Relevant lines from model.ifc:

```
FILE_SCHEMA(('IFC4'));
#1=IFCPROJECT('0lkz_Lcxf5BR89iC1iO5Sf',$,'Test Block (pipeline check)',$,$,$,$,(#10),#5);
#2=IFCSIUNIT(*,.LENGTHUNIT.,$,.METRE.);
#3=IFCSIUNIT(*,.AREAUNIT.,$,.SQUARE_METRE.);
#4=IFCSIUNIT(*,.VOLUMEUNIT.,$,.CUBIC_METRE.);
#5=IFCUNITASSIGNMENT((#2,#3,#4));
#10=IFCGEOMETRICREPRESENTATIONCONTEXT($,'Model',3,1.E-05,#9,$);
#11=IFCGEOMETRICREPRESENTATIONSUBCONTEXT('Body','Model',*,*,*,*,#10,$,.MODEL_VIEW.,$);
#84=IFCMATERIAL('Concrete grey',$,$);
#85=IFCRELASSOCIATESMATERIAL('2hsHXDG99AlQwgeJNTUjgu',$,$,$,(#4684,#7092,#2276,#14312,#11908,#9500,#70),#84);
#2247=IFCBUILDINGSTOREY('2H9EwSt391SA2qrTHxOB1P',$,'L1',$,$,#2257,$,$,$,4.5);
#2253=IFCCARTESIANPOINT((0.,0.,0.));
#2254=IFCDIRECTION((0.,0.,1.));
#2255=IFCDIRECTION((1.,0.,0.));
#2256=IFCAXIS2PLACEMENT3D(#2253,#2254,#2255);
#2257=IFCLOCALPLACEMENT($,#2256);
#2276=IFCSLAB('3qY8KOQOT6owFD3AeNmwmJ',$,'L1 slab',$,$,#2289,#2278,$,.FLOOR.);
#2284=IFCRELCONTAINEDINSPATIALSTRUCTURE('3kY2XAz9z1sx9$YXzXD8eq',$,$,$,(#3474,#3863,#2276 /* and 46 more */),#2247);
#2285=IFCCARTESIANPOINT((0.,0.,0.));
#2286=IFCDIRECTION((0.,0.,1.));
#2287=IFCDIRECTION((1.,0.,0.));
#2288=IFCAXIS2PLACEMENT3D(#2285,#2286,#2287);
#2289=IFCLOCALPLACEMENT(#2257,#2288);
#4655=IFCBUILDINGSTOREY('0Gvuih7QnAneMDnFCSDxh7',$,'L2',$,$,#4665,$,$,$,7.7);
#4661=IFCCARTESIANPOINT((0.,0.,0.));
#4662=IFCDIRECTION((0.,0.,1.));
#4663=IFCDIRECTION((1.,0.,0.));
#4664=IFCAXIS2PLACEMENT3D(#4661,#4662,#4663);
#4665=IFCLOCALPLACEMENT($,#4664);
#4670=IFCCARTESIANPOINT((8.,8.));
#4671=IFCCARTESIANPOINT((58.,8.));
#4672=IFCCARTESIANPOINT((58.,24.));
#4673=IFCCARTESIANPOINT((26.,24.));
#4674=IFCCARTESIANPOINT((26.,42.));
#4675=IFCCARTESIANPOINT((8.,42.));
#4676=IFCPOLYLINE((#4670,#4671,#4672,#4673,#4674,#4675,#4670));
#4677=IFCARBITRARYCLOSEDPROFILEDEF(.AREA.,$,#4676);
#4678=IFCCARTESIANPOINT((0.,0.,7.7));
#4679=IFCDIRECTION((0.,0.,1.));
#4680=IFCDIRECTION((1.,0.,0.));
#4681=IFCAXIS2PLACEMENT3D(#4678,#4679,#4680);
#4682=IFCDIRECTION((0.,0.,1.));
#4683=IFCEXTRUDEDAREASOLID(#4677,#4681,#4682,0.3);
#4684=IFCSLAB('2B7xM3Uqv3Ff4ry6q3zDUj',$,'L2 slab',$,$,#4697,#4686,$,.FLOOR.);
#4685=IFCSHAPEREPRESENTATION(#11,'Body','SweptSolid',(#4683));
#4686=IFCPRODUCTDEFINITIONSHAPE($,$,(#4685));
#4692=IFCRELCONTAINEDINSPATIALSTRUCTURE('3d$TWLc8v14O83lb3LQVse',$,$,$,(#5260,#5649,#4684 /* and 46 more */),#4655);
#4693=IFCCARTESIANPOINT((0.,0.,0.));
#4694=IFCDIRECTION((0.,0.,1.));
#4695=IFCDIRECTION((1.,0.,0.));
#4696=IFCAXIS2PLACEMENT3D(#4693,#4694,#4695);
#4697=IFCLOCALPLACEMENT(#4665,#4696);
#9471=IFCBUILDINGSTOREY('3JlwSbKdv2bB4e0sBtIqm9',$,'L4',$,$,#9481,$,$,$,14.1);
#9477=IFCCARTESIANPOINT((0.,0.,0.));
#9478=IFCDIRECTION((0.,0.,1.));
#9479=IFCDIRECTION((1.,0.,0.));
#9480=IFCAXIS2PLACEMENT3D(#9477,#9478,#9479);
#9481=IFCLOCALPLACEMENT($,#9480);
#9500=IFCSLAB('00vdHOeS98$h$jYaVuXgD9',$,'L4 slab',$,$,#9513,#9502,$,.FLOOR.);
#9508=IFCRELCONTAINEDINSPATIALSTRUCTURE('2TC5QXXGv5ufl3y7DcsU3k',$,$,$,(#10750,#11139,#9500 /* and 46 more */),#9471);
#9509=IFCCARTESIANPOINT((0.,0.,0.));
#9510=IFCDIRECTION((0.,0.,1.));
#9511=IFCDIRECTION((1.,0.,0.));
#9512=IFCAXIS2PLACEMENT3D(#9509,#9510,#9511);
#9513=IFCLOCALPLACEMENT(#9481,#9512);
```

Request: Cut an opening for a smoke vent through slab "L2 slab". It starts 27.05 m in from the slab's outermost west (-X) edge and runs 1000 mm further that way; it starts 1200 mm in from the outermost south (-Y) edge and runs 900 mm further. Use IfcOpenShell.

```python
import numpy as np
import ifcopenshell
import ifcopenshell.api.feature
import ifcopenshell.api.geometry
import ifcopenshell.api.root
import ifcopenshell.geom
import ifcopenshell.util.placement
import ifcopenshell.util.representation
import ifcopenshell.util.shape
import ifcopenshell.util.unit

model = ifcopenshell.open("model.ifc")
unit_scale = ifcopenshell.util.unit.calculate_unit_scale(model)
settings = ifcopenshell.geom.settings()


def volume(element):
    """Net volume in cubic metres, openings subtracted."""
    shape = ifcopenshell.geom.create_shape(settings, element)
    return ifcopenshell.util.shape.get_volume(shape.geometry)


slab = model.by_guid("2B7xM3Uqv3Ff4ry6q3zDUj")
before = volume(slab)

# Extent in the slab's own axes, in metres. The edges named are its -X and -Y sides.
slab_shape = ifcopenshell.geom.create_shape(settings, slab)
vertices = ifcopenshell.util.shape.get_vertices(slab_shape.geometry)
x_min, y_min, bottom = vertices.min(axis=0)
top = vertices[:, 2].max()

opening = ifcopenshell.api.root.create_entity(model, ifc_class="IfcOpeningElement", name="Smoke vent opening", predefined_type="OPENING")
context = ifcopenshell.util.representation.get_context(model, "Model", "Body", "MODEL_VIEW")
width, depth = 1, 0.9
outline = [(0.0, 0.0), (width, 0.0), (width, depth), (0.0, depth), (0.0, 0.0)]
# Overshoot both faces by 50 mm so the cut is clean.
shape = ifcopenshell.api.geometry.add_slab_representation(
    model, context=context, depth=top - bottom + 0.1, polyline=outline
)
ifcopenshell.api.geometry.assign_representation(model, product=opening, representation=shape)

matrix = ifcopenshell.util.placement.get_local_placement(slab.ObjectPlacement)
matrix[:, 3] = matrix @ np.append(np.array([x_min + 27.05, y_min + 1.2, bottom - 0.05]) / unit_scale, 1.0)
ifcopenshell.api.geometry.edit_object_placement(model, product=opening, matrix=matrix, is_si=False)
ifcopenshell.api.feature.add_feature(model, feature=opening, element=slab)

after = volume(slab)

print(f"slab volume {before:.3f} -> {after:.3f} m3")

model.write("model_edited.ifc")
```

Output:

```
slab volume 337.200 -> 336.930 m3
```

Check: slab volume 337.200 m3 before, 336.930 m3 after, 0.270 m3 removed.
